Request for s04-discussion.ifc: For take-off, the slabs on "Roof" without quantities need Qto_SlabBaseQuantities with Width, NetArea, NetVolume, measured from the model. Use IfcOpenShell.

First a look at what the model holds.

```python
import ifcopenshell
import ifcopenshell.util.element
import ifcopenshell.util.unit

model = ifcopenshell.open("s04-discussion.ifc")
print(model.schema)
for unit_type in ("LENGTHUNIT", "AREAUNIT", "VOLUMEUNIT"):
    print(unit_type, ifcopenshell.util.unit.calculate_unit_scale(model, unit_type))
storey = next(s for s in model.by_type("IfcBuildingStorey") if s.Name == "Roof")
slabs = [e for e in ifcopenshell.util.element.get_decomposition(storey) if e.is_a("IfcSlab")]
for e in sorted(slabs, key=lambda e: e.id()):
    print(e.id(), e.is_a(), e.Name, list(ifcopenshell.util.element.get_psets(e, qtos_only=True)), sep=" | ")
```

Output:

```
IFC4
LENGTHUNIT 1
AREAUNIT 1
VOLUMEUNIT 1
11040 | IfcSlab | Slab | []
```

```python
import ifcopenshell
import ifcopenshell.api.pset
import ifcopenshell.geom
import ifcopenshell.util.element
import ifcopenshell.util.shape
import ifcopenshell.util.unit

model = ifcopenshell.open("s04-discussion.ifc")
unit_scale = ifcopenshell.util.unit.calculate_unit_scale(model)
area_scale = ifcopenshell.util.unit.calculate_unit_scale(model, "AREAUNIT")
volume_scale = ifcopenshell.util.unit.calculate_unit_scale(model, "VOLUMEUNIT")
settings = ifcopenshell.geom.settings()

storey = next(s for s in model.by_type("IfcBuildingStorey") if s.Name == "Roof")
slabs = [e for e in ifcopenshell.util.element.get_decomposition(storey) if e.is_a("IfcSlab")]

for e in sorted(slabs, key=lambda e: e.id()):
    if ifcopenshell.util.element.get_psets(e, qtos_only=True, should_inherit=False):
        continue
    # Geometry comes back in metres, in the element's own axes.
    shape = ifcopenshell.geom.create_shape(settings, e)
    values = {
        "Width": ifcopenshell.util.shape.get_z(shape.geometry) / unit_scale,
        "NetArea": ifcopenshell.util.shape.get_footprint_area(shape.geometry) / area_scale,
        "NetVolume": ifcopenshell.util.shape.get_volume(shape.geometry) / volume_scale,
    }
    qto = ifcopenshell.api.pset.add_qto(model, product=e, name="Qto_SlabBaseQuantities")
    ifcopenshell.api.pset.edit_qto(model, qto=qto, properties=values)
    print(e.id(), {k: round(v, 3) for k, v in values.items()})

model.write("s04-discussion_updated.ifc")
```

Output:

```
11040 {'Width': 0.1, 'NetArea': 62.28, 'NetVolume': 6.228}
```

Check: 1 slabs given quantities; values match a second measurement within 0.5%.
